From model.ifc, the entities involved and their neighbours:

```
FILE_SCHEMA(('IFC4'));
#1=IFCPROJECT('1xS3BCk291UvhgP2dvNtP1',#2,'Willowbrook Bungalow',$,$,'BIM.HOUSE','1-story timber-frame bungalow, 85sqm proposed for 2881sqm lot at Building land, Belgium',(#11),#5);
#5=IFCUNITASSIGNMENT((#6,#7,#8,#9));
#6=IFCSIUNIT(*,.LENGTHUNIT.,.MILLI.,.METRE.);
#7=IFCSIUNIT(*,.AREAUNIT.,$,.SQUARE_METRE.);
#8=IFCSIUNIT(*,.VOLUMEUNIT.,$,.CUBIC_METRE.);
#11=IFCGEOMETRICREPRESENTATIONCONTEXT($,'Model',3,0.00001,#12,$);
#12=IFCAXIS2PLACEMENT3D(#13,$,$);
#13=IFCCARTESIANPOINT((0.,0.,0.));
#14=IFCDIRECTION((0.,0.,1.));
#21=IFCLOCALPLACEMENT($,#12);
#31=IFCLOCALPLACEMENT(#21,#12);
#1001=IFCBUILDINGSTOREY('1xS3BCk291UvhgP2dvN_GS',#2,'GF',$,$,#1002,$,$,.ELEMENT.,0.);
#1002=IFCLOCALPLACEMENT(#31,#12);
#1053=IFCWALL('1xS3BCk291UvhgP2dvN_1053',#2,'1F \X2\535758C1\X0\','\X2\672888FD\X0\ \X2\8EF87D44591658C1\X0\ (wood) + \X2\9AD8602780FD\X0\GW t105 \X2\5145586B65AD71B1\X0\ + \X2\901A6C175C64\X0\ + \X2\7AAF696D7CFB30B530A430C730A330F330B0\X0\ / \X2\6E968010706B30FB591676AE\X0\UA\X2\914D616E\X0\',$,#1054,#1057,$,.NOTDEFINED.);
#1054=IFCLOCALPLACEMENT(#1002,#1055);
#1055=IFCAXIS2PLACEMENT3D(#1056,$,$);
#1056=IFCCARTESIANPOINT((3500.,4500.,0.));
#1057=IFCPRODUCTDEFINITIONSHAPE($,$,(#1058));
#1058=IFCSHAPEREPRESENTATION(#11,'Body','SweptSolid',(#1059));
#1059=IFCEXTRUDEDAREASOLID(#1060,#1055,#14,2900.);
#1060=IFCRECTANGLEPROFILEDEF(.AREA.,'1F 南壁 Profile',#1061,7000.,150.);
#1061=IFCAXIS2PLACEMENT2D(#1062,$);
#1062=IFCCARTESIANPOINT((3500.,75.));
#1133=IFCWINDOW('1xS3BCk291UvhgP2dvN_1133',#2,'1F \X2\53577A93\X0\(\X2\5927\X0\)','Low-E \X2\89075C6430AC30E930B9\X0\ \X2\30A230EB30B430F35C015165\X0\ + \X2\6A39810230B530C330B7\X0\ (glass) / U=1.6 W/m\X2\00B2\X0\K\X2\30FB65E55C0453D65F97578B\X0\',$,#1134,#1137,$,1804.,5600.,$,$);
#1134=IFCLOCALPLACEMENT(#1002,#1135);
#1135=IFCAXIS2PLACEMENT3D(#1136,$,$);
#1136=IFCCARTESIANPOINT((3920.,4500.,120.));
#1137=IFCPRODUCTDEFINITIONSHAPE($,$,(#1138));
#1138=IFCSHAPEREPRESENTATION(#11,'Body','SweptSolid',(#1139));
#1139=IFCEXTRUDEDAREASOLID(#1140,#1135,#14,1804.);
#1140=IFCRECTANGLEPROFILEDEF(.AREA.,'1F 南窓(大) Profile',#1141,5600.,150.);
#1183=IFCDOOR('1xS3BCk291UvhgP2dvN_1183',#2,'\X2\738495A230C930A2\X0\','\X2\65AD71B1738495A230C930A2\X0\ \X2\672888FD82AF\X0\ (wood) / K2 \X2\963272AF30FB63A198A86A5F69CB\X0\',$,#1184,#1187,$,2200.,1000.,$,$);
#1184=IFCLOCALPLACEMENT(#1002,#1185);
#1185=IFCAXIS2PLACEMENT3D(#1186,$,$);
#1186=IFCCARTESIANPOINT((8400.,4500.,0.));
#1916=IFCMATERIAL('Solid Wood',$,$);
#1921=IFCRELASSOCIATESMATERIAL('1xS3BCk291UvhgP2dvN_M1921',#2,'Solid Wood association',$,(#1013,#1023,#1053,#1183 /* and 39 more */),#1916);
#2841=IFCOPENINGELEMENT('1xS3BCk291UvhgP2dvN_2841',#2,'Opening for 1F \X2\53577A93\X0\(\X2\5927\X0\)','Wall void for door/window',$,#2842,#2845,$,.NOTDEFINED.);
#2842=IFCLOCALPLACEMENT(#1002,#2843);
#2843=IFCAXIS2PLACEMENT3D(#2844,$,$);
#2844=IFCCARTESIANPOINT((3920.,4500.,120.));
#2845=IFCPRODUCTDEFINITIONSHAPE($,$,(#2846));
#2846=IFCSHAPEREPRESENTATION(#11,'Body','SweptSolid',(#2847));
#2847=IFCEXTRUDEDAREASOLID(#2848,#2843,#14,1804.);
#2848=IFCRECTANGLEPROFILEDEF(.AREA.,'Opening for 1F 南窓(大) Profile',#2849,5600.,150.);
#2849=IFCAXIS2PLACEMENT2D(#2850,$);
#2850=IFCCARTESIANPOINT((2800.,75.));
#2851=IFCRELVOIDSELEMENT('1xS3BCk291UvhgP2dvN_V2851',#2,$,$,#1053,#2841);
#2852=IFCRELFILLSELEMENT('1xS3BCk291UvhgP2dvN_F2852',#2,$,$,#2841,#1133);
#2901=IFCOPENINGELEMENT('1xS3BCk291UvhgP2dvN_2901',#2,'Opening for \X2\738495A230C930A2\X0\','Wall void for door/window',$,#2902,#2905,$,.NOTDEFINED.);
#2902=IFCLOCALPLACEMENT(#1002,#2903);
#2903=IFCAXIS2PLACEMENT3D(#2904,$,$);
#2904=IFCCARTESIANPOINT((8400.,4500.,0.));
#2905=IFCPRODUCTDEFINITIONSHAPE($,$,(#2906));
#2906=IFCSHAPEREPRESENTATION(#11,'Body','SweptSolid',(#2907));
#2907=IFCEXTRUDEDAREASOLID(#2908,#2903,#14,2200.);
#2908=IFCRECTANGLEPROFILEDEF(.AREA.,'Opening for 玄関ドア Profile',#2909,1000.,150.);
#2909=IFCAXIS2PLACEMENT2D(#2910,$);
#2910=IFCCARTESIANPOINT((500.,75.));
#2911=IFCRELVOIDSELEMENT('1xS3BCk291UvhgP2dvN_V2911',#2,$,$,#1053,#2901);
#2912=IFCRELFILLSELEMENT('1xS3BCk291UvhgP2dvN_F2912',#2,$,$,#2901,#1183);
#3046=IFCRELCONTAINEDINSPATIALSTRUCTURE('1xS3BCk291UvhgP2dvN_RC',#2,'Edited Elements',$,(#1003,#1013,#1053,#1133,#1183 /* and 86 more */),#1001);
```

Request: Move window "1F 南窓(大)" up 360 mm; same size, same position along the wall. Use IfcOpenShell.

```python
import numpy as np
import ifcopenshell
import ifcopenshell.api.geometry
import ifcopenshell.util.placement
import ifcopenshell.util.unit

model = ifcopenshell.open("model.ifc")
unit_scale = ifcopenshell.util.unit.calculate_unit_scale(model)

window = model.by_guid("1xS3BCk291UvhgP2dvN_1133")
opening = window.FillsVoids[0].RelatingOpeningElement
dz = 0.36 / unit_scale

shift = np.array([0.0, 0.0, dz])
# The window is not placed relative to its opening, so move both.
for product in (opening, window):
    matrix = ifcopenshell.util.placement.get_local_placement(product.ObjectPlacement)
    matrix[:3, 3] += shift
    ifcopenshell.api.geometry.edit_object_placement(model, product=product, matrix=matrix, is_si=False)

print(f"moved by {dz * unit_scale:+.3f} m")

model.write("model-out.ifc")
```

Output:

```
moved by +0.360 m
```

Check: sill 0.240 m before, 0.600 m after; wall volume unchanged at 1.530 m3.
